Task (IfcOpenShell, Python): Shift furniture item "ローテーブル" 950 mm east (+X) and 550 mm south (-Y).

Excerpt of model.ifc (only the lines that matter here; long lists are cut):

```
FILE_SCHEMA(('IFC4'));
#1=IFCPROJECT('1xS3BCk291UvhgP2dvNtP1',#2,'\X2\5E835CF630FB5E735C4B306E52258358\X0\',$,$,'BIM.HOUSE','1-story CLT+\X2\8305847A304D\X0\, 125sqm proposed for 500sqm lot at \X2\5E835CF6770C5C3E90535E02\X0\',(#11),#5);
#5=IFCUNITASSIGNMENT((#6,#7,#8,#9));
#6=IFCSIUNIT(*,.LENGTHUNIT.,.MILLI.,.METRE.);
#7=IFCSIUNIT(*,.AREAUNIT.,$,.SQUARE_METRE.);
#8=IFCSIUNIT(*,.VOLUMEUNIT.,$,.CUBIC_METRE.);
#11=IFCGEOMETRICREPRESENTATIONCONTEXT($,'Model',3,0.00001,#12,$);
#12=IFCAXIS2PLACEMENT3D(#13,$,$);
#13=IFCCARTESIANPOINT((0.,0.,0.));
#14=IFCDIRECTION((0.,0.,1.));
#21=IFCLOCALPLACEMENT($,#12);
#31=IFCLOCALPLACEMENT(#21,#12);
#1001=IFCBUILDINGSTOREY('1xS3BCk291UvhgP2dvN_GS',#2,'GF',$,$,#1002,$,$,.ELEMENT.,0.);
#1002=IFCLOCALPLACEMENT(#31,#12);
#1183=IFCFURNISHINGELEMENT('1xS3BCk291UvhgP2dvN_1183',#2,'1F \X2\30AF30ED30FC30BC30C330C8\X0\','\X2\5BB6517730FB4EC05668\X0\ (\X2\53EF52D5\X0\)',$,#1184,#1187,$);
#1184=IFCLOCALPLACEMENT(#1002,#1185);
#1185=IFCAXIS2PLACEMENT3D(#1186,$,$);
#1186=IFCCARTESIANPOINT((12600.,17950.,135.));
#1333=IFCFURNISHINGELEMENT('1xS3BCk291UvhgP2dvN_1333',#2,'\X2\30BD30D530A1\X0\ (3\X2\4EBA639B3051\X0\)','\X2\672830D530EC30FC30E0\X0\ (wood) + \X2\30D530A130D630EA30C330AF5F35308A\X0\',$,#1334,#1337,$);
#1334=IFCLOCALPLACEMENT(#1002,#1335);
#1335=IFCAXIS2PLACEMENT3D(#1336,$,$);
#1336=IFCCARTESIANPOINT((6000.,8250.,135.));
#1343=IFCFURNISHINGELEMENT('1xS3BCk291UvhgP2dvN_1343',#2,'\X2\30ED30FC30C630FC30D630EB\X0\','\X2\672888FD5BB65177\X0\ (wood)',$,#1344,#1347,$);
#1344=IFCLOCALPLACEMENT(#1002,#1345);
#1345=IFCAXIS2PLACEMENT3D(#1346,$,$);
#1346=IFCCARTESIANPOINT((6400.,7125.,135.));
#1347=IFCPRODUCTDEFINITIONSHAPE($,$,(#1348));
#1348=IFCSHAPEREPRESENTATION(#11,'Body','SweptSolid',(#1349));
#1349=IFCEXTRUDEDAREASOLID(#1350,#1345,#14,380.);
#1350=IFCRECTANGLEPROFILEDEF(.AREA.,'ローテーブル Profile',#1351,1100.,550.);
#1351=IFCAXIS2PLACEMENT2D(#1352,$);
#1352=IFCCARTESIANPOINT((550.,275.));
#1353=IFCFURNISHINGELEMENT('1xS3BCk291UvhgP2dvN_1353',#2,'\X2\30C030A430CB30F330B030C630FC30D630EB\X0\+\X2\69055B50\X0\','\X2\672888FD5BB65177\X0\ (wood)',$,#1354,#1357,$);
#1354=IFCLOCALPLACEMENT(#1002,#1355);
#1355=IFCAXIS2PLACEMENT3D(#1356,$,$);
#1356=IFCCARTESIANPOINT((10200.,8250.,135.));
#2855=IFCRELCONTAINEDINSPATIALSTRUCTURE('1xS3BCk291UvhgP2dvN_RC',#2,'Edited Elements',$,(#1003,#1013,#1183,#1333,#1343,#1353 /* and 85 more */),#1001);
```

```python
import ifcopenshell
import ifcopenshell.api.geometry
import ifcopenshell.util.placement
import ifcopenshell.util.unit

model = ifcopenshell.open("model.ifc")
unit_scale = ifcopenshell.util.unit.calculate_unit_scale(model)

item = model.by_guid("1xS3BCk291UvhgP2dvN_1343")
matrix = ifcopenshell.util.placement.get_local_placement(item.ObjectPlacement)
matrix[0, 3] += 0.95 / unit_scale
matrix[1, 3] -= 0.55 / unit_scale
ifcopenshell.api.geometry.edit_object_placement(model, product=item, matrix=matrix, is_si=False)

print(ifcopenshell.util.placement.get_local_placement(item.ObjectPlacement).round(3) + 0.0)

model.write("model_edited.ifc")
```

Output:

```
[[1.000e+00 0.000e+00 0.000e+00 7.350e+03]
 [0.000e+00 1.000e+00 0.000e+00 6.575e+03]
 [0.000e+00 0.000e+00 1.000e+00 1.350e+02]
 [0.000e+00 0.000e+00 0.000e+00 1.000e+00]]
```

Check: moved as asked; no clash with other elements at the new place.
